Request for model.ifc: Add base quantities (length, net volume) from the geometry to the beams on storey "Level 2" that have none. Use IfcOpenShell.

First a look at what the model holds.

```python
import ifcopenshell
import ifcopenshell.util.element
import ifcopenshell.util.unit

model = ifcopenshell.open("model.ifc")
print(model.schema)
for unit_type in ("LENGTHUNIT", "AREAUNIT", "VOLUMEUNIT"):
    print(unit_type, ifcopenshell.util.unit.calculate_unit_scale(model, unit_type))
storey = next(s for s in model.by_type("IfcBuildingStorey") if s.Name == "Level 2")
beams = [e for e in ifcopenshell.util.element.get_decomposition(storey) if e.is_a("IfcBeam")]
for e in sorted(beams, key=lambda e: e.id()):
    print(e.id(), e.is_a(), e.Name, list(ifcopenshell.util.element.get_psets(e, qtos_only=True)), sep=" | ")
```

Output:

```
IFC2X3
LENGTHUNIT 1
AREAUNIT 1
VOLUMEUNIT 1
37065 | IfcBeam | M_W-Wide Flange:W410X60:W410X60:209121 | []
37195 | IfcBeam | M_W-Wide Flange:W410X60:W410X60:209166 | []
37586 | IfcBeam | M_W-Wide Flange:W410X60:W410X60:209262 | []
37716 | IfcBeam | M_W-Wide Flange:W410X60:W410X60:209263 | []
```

```python
import ifcopenshell
import ifcopenshell.api.pset
import ifcopenshell.geom
import ifcopenshell.util.element
import ifcopenshell.util.shape
import ifcopenshell.util.unit

model = ifcopenshell.open("model.ifc")
unit_scale = ifcopenshell.util.unit.calculate_unit_scale(model)
volume_scale = ifcopenshell.util.unit.calculate_unit_scale(model, "VOLUMEUNIT")
settings = ifcopenshell.geom.settings()

storey = next(s for s in model.by_type("IfcBuildingStorey") if s.Name == "Level 2")
beams = [e for e in ifcopenshell.util.element.get_decomposition(storey) if e.is_a("IfcBeam")]

for e in sorted(beams, key=lambda e: e.id()):
    if ifcopenshell.util.element.get_psets(e, qtos_only=True, should_inherit=False):
        continue
    # Geometry comes back in metres, in the element's own axes.
    shape = ifcopenshell.geom.create_shape(settings, e)
    values = {
        "Length": ifcopenshell.util.shape.get_max_xyz(shape.geometry) / unit_scale,
        "NetVolume": ifcopenshell.util.shape.get_volume(shape.geometry) / volume_scale,
    }
    qto = ifcopenshell.api.pset.add_qto(model, product=e, name="BaseQuantities")
    ifcopenshell.api.pset.edit_qto(model, qto=qto, properties=values)
    print(e.id(), {k: round(v, 3) for k, v in values.items()})

model.write("model_v2.ifc")
```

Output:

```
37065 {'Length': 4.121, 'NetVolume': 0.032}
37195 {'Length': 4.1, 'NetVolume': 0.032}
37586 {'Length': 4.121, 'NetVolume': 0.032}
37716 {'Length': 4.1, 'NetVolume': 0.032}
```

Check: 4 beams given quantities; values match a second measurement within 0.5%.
